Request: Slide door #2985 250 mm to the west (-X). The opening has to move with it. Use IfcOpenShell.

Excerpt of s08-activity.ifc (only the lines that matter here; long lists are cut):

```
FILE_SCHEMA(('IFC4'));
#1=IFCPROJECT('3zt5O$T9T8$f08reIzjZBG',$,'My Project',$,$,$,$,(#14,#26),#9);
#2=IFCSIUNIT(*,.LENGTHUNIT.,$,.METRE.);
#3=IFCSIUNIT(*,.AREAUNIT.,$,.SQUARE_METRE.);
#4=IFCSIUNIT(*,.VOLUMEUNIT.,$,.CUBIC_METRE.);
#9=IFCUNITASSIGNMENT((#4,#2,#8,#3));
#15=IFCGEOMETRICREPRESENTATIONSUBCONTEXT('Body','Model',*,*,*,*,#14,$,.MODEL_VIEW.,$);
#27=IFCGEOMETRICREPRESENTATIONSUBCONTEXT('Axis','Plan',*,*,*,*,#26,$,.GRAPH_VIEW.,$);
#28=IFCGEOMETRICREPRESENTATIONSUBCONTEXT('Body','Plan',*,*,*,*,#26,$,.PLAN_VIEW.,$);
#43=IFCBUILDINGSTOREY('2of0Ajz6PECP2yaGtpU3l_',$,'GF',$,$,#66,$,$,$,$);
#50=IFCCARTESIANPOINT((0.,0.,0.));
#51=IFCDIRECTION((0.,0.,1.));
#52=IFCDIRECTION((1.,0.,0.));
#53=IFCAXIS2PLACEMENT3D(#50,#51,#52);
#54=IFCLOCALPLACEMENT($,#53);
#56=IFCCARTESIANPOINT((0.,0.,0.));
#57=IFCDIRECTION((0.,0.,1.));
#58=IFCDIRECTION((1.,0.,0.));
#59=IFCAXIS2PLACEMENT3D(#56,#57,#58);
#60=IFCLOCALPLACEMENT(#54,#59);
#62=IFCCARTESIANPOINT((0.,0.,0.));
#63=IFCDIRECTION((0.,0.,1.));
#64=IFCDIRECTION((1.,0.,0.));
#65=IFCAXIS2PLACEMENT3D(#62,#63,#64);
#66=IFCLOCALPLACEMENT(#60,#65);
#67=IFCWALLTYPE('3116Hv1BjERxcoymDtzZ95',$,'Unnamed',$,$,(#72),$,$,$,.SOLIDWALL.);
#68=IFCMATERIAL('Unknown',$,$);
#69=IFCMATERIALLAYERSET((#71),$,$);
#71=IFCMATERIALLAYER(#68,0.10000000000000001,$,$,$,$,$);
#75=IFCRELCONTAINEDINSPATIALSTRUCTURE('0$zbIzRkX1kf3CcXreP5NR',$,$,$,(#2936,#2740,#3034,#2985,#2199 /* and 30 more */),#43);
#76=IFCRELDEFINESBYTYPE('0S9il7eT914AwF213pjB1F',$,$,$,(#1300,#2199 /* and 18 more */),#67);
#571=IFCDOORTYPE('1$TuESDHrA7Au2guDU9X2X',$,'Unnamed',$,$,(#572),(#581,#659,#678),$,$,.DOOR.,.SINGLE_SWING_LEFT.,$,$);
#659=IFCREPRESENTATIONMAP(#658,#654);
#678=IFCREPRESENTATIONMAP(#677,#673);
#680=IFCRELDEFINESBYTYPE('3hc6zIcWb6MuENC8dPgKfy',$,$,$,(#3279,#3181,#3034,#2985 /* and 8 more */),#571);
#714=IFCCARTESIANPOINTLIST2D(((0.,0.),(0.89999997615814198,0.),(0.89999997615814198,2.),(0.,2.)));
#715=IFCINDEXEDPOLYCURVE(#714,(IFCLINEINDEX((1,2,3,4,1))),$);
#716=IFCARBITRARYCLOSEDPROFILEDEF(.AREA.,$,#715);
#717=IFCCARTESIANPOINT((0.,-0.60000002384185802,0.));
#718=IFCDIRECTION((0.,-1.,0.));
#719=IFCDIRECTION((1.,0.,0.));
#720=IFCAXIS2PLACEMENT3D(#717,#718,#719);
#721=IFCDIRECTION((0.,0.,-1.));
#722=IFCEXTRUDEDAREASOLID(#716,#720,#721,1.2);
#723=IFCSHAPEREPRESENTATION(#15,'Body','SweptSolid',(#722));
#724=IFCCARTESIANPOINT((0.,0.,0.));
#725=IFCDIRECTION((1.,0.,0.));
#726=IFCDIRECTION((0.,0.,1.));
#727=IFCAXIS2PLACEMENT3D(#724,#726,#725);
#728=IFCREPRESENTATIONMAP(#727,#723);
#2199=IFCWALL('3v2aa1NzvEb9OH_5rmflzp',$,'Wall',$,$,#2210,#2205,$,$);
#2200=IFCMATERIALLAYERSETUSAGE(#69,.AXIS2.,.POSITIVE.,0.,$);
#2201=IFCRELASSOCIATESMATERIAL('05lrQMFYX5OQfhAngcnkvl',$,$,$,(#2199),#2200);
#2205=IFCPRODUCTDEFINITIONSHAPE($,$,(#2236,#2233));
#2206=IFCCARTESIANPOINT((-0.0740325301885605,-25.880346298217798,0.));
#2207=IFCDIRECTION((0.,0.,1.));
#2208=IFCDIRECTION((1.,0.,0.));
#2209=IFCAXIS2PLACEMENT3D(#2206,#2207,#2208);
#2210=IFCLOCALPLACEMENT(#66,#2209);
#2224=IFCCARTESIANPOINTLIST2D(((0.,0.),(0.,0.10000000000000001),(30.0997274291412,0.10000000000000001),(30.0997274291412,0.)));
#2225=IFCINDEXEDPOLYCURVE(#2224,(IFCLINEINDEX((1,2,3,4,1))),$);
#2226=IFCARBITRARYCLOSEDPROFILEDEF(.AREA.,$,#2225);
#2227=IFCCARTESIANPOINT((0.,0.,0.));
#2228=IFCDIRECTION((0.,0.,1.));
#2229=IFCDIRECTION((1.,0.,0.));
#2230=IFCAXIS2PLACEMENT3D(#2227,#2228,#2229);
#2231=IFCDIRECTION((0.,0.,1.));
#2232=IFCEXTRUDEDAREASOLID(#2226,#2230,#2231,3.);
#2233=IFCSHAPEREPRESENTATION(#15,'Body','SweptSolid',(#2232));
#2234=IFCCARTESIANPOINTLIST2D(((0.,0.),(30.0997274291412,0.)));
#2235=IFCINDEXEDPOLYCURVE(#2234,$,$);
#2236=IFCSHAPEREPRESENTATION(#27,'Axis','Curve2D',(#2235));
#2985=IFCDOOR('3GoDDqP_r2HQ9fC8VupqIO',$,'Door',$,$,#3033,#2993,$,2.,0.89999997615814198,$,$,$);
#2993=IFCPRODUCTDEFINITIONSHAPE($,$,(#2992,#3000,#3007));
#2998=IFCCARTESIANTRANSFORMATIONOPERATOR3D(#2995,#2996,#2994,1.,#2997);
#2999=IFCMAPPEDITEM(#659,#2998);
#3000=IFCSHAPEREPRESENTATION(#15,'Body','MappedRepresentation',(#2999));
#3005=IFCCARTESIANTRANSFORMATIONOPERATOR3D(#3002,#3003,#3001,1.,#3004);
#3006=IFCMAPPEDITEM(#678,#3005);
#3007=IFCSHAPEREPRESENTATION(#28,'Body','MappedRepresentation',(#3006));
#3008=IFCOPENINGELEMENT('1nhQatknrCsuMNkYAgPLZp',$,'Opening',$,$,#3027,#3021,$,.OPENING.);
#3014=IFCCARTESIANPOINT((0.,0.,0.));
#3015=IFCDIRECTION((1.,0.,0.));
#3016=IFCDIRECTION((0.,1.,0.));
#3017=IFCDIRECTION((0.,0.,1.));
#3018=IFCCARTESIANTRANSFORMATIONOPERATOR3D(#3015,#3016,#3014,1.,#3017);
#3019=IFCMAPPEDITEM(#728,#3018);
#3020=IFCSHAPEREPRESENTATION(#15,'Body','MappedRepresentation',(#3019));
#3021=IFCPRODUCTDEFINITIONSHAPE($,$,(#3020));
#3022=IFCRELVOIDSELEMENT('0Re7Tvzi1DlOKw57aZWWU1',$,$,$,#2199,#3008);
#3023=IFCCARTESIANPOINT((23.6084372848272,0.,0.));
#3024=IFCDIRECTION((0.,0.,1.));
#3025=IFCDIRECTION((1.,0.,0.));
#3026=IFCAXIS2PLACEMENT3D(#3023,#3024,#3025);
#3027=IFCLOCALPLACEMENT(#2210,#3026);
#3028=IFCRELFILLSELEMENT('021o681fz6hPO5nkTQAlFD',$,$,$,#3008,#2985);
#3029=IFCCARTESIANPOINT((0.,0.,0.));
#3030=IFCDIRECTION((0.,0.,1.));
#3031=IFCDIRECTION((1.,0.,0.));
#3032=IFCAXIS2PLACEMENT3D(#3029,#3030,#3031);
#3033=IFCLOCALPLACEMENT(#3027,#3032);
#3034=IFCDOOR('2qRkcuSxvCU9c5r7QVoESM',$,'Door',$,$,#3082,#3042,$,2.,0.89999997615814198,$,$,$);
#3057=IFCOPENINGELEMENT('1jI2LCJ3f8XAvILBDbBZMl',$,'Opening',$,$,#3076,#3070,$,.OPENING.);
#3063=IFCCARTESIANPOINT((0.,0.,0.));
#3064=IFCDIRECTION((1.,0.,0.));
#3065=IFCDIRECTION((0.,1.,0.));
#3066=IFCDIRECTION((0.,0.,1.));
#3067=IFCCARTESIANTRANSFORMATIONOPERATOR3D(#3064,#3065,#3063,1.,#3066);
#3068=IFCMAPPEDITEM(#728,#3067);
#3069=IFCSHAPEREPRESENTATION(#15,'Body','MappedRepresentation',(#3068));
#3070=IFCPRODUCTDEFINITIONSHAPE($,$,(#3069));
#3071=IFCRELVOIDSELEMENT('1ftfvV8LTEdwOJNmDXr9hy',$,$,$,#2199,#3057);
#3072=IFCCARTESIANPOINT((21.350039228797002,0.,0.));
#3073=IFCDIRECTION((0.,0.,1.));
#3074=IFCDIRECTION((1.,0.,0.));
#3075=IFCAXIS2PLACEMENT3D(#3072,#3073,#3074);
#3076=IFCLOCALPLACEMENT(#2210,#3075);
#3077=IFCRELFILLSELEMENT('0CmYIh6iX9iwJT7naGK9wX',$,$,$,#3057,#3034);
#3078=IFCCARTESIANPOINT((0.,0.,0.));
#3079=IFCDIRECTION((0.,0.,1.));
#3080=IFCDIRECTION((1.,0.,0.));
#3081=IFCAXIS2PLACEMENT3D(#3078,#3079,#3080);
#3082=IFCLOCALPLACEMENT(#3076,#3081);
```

```python
import ifcopenshell
import ifcopenshell.api.geometry
import ifcopenshell.util.placement

model = ifcopenshell.open("s08-activity.ifc")

door = model.by_id(2985)
opening = door.FillsVoids[0].RelatingOpeningElement
wall = opening.VoidsElements[0].RelatingBuildingElement

wall_matrix = ifcopenshell.util.placement.get_local_placement(wall.ObjectPlacement)
shift = wall_matrix[:3, 0] * -0.25
before = ifcopenshell.util.placement.get_local_placement(door.ObjectPlacement)[:3, 3].copy()

# The door is placed relative to its opening, so it follows when the opening moves.
matrix = ifcopenshell.util.placement.get_local_placement(opening.ObjectPlacement)
matrix[:3, 3] += shift
ifcopenshell.api.geometry.edit_object_placement(
    model, product=opening, matrix=matrix, is_si=False, should_transform_children=True
)

after = ifcopenshell.util.placement.get_local_placement(door.ObjectPlacement)[:3, 3]
print("door moved by", (after - before).round(3) + 0.0)

model.write("s08-activity_v2.ifc")
```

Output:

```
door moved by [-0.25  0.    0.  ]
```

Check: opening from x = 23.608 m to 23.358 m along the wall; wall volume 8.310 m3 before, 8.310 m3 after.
